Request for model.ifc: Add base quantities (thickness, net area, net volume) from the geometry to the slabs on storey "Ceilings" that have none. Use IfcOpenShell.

First a look at what the model holds.

```python
import ifcopenshell
import ifcopenshell.util.element
import ifcopenshell.util.unit

model = ifcopenshell.open("model.ifc")
print(model.schema)
for unit_type in ("LENGTHUNIT", "AREAUNIT", "VOLUMEUNIT"):
    print(unit_type, ifcopenshell.util.unit.calculate_unit_scale(model, unit_type))
storey = next(s for s in model.by_type("IfcBuildingStorey") if s.Name == "Ceilings")
slabs = [e for e in ifcopenshell.util.element.get_decomposition(storey) if e.is_a("IfcSlab")]
for e in sorted(slabs, key=lambda e: e.id()):
    print(e.id(), e.is_a(), e.Name, list(ifcopenshell.util.element.get_psets(e, qtos_only=True)), sep=" | ")
```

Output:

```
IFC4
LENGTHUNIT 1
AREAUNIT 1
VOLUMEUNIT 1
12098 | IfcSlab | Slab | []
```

```python
import ifcopenshell
import ifcopenshell.api.pset
import ifcopenshell.geom
import ifcopenshell.util.element
import ifcopenshell.util.shape
import ifcopenshell.util.unit

model = ifcopenshell.open("model.ifc")
unit_scale = ifcopenshell.util.unit.calculate_unit_scale(model)
area_scale = ifcopenshell.util.unit.calculate_unit_scale(model, "AREAUNIT")
volume_scale = ifcopenshell.util.unit.calculate_unit_scale(model, "VOLUMEUNIT")
settings = ifcopenshell.geom.settings()

storey = next(s for s in model.by_type("IfcBuildingStorey") if s.Name == "Ceilings")
slabs = [e for e in ifcopenshell.util.element.get_decomposition(storey) if e.is_a("IfcSlab")]

for e in sorted(slabs, key=lambda e: e.id()):
    if ifcopenshell.util.element.get_psets(e, qtos_only=True, should_inherit=False):
        continue
    # Geometry comes back in metres, in the element's own axes.
    shape = ifcopenshell.geom.create_shape(settings, e)
    values = {
        "Width": ifcopenshell.util.shape.get_z(shape.geometry) / unit_scale,
        "NetArea": ifcopenshell.util.shape.get_footprint_area(shape.geometry) / area_scale,
        "NetVolume": ifcopenshell.util.shape.get_volume(shape.geometry) / volume_scale,
    }
    qto = ifcopenshell.api.pset.add_qto(model, product=e, name="Qto_SlabBaseQuantities")
    ifcopenshell.api.pset.edit_qto(model, qto=qto, properties=values)
    print(e.id(), {k: round(v, 3) for k, v in values.items()})

model.write("model_updated.ifc")
```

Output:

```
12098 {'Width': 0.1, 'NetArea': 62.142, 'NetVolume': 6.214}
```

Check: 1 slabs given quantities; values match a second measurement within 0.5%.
